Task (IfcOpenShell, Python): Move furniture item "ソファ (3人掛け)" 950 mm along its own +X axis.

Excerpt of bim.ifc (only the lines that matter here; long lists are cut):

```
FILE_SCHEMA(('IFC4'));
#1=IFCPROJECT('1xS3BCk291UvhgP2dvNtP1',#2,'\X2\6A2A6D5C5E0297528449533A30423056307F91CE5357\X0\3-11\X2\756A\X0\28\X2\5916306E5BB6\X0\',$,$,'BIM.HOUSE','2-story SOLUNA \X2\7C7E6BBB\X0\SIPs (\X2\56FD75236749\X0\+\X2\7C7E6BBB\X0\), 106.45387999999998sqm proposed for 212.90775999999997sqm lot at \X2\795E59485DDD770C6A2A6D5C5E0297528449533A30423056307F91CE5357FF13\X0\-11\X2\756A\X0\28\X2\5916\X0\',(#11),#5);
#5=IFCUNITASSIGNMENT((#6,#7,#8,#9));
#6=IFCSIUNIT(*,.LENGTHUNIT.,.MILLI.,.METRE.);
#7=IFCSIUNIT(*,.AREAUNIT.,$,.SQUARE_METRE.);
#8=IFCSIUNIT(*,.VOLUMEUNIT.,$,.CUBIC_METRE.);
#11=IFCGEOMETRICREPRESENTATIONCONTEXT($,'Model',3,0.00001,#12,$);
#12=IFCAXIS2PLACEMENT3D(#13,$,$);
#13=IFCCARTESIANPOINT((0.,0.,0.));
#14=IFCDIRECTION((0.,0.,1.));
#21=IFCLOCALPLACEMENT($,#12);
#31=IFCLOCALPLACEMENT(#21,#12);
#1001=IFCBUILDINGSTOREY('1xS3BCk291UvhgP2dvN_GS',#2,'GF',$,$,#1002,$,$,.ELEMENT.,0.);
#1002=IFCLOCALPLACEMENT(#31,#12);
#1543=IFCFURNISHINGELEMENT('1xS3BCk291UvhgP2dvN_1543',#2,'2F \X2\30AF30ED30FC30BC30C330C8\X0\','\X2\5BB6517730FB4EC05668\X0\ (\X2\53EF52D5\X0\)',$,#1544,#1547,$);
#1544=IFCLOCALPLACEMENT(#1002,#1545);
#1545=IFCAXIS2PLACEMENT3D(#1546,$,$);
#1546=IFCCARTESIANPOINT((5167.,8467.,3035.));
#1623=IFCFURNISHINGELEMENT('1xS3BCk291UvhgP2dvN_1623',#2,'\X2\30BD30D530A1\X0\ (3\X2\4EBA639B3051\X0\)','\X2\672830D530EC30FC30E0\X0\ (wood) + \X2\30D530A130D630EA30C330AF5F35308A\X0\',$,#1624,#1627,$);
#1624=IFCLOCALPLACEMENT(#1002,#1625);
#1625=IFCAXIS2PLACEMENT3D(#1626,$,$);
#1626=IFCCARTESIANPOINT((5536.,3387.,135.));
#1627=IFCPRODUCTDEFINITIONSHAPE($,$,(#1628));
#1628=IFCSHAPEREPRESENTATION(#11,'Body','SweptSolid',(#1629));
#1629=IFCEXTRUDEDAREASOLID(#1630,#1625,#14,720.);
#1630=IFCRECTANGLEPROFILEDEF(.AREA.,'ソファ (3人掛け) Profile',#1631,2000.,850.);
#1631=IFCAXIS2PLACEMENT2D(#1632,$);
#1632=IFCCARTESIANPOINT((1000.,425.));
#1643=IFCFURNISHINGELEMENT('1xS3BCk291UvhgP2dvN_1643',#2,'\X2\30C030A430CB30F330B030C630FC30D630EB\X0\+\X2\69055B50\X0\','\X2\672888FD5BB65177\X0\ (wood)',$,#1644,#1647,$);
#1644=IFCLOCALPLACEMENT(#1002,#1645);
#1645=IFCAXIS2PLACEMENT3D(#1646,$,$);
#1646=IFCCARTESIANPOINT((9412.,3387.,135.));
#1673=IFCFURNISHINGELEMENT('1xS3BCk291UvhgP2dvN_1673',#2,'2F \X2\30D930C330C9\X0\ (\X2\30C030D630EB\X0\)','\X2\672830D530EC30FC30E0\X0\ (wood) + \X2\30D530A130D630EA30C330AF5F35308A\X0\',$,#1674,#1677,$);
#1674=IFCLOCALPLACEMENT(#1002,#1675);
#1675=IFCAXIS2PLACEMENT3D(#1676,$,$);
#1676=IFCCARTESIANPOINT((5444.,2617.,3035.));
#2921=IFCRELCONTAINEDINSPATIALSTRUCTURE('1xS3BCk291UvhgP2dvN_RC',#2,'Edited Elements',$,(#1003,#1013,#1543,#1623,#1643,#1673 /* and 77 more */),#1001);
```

```python
import ifcopenshell
import ifcopenshell.api.geometry
import ifcopenshell.util.placement

model = ifcopenshell.open("bim.ifc")

item = model.by_guid("1xS3BCk291UvhgP2dvN_1623")
matrix = ifcopenshell.util.placement.get_local_placement(item.ObjectPlacement)
matrix[:3, 3] += matrix[:3, 0] * 950.0
ifcopenshell.api.geometry.edit_object_placement(model, product=item, matrix=matrix, is_si=False)

print(ifcopenshell.util.placement.get_local_placement(item.ObjectPlacement).round(3) + 0.0)

model.write("bim-out.ifc")
```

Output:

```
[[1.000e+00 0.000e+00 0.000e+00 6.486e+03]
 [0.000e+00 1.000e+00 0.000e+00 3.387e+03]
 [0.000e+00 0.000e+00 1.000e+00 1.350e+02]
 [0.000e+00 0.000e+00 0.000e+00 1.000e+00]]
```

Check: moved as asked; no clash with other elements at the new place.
